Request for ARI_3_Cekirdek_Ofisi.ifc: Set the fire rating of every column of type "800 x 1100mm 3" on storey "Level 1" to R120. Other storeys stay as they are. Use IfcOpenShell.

First a look at what the model holds.

```python
import ifcopenshell
import ifcopenshell.util.element

model = ifcopenshell.open("ARI_3_Cekirdek_Ofisi.ifc")
print(model.schema)
storey = next(s for s in model.by_type("IfcBuildingStorey") if s.Name == "Level 1")
columns = [e for e in ifcopenshell.util.element.get_decomposition(storey) if e.is_a("IfcColumn")]
seen = {}
for e in columns:
    element_type = ifcopenshell.util.element.get_type(e)
    key = (element_type.Name if element_type != e and element_type else None, ifcopenshell.util.element.get_pset(e, "Pset_ColumnCommon", "FireRating"))
    seen[key] = seen.get(key, 0) + 1
for (name, value), count in sorted(seen.items(), key=str):
    print(count, "x", name, "|", value)
```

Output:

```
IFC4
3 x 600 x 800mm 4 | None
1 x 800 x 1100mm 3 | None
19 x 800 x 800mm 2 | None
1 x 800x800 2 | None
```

```python
import ifcopenshell
import ifcopenshell.api.pset
import ifcopenshell.util.element

model = ifcopenshell.open("ARI_3_Cekirdek_Ofisi.ifc")

storey = next(s for s in model.by_type("IfcBuildingStorey") if s.Name == "Level 1")
columns = [e for e in ifcopenshell.util.element.get_decomposition(storey) if e.is_a("IfcColumn")]

count = 0
for e in columns:
    element_type = ifcopenshell.util.element.get_type(e)
    if element_type in (None, e) or element_type.Name != "800 x 1100mm 3":
        continue
    # add_pset returns the element's existing set when there is one.
    pset = ifcopenshell.api.pset.add_pset(model, product=e, name="Pset_ColumnCommon")
    ifcopenshell.api.pset.edit_pset(model, pset=pset, properties={"FireRating": "R120"})
    count += 1

print(count, "columns updated")

model.write("ARI_3_Cekirdek_Ofisi_edited.ifc")
```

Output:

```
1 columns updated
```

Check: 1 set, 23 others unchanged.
